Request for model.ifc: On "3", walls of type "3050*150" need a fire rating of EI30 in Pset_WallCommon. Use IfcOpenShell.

First a look at what the model holds.

```python
import ifcopenshell
import ifcopenshell.util.element

model = ifcopenshell.open("model.ifc")
print(model.schema)
storey = next(s for s in model.by_type("IfcBuildingStorey") if s.Name == "3")
walls = [e for e in ifcopenshell.util.element.get_decomposition(storey) if e.is_a("IfcWall")]
seen = {}
for e in walls:
    element_type = ifcopenshell.util.element.get_type(e)
    key = (element_type.Name if element_type != e and element_type else None, ifcopenshell.util.element.get_pset(e, "Pset_WallCommon", "FireRating"))
    seen[key] = seen.get(key, 0) + 1
for (name, value), count in sorted(seen.items(), key=str):
    print(count, "x", name, "|", value)
```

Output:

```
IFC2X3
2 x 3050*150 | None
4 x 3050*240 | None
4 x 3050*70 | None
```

```python
import ifcopenshell
import ifcopenshell.api.pset
import ifcopenshell.util.element

model = ifcopenshell.open("model.ifc")

storey = next(s for s in model.by_type("IfcBuildingStorey") if s.Name == "3")
walls = [e for e in ifcopenshell.util.element.get_decomposition(storey) if e.is_a("IfcWall")]

count = 0
for e in walls:
    element_type = ifcopenshell.util.element.get_type(e)
    if element_type in (None, e) or element_type.Name != "3050*150":
        continue
    # add_pset returns the element's existing set when there is one.
    pset = ifcopenshell.api.pset.add_pset(model, product=e, name="Pset_WallCommon")
    ifcopenshell.api.pset.edit_pset(model, pset=pset, properties={"FireRating": "EI30"})
    count += 1

print(count, "walls updated")

model.write("model-out.ifc")
```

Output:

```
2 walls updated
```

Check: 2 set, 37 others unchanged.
